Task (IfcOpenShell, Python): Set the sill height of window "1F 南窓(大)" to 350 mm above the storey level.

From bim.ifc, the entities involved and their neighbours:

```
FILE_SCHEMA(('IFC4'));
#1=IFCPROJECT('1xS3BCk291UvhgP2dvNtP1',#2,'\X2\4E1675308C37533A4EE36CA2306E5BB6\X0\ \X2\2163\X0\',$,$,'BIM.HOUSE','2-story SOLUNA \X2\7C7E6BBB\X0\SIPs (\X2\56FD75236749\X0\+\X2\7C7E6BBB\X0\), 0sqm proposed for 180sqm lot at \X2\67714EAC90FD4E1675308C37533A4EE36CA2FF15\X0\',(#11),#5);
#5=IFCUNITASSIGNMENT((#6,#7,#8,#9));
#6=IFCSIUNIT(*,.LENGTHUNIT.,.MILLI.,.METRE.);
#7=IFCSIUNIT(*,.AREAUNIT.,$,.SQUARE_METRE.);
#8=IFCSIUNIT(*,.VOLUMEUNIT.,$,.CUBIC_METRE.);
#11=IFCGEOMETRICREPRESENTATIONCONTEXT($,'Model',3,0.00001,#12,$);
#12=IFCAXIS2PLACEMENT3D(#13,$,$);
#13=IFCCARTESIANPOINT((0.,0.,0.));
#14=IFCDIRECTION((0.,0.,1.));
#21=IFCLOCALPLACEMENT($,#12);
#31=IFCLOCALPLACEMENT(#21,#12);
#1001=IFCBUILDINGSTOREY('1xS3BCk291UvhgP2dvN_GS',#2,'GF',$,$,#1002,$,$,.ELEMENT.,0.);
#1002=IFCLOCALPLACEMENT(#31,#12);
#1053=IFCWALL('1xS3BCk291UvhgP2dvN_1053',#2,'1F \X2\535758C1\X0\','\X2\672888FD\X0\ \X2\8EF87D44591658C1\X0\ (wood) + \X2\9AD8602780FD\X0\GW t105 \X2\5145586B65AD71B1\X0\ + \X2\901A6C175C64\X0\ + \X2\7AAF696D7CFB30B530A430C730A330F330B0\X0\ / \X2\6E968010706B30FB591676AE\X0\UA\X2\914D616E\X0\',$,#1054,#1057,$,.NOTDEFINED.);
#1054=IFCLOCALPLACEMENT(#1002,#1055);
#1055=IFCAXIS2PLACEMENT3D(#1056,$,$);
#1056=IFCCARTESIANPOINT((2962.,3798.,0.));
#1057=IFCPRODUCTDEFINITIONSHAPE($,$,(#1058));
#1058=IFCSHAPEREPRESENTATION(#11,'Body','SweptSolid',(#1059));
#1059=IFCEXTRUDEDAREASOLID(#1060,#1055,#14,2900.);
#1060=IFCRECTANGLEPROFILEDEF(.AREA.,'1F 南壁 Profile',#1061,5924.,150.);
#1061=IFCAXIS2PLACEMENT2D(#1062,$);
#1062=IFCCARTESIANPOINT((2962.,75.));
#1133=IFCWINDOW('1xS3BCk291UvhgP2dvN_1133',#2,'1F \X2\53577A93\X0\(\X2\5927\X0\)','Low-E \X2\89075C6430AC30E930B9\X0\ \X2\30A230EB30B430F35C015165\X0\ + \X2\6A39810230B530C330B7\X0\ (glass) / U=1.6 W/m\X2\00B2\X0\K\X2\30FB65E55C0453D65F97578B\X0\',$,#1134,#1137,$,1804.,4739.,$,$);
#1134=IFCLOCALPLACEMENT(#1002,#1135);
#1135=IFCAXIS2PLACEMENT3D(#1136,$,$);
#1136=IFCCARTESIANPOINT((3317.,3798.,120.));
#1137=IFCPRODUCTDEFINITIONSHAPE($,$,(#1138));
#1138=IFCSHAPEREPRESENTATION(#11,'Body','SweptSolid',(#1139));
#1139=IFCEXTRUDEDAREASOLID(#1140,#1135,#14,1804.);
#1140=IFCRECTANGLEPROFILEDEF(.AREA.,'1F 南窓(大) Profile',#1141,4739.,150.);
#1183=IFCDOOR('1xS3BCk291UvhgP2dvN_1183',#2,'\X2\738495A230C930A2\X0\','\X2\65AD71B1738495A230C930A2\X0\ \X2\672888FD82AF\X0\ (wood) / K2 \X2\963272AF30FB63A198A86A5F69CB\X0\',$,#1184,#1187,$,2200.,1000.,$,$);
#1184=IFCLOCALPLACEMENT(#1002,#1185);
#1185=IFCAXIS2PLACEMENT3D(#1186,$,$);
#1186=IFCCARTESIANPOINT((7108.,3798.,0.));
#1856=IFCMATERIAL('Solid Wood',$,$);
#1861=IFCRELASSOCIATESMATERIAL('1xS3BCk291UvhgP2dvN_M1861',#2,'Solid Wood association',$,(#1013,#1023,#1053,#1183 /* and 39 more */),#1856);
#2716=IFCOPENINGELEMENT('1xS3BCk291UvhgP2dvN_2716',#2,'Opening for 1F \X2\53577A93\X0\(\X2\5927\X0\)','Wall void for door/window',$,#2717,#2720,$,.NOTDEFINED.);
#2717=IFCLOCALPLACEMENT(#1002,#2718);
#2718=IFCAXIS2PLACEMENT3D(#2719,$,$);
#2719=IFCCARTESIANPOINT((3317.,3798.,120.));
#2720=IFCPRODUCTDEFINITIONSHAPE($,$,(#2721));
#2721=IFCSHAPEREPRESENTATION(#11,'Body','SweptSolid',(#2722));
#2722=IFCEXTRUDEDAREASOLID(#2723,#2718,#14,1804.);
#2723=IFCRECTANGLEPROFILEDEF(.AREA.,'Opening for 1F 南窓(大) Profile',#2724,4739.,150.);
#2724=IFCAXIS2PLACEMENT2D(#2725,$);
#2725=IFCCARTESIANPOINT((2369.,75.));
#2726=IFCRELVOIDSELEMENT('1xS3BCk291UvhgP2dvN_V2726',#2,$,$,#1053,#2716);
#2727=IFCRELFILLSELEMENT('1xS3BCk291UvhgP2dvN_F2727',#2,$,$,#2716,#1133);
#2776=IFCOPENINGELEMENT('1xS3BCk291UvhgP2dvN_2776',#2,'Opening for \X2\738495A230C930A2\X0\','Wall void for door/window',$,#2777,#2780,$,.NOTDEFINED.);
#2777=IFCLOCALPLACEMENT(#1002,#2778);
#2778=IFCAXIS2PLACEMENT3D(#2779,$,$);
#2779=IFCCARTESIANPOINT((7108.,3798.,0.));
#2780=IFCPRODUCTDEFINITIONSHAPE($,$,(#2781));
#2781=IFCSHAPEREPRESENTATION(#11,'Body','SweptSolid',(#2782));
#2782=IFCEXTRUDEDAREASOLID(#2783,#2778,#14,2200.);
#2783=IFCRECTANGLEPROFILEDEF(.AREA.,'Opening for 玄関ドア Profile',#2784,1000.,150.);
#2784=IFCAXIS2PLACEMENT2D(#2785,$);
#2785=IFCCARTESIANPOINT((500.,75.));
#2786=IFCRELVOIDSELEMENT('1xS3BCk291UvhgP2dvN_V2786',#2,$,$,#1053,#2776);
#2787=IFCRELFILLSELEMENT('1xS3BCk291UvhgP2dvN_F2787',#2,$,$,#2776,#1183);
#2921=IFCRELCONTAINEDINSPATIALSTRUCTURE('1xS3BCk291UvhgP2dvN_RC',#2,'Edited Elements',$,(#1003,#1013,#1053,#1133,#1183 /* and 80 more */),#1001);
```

```python
import numpy as np
import ifcopenshell
import ifcopenshell.api.geometry
import ifcopenshell.geom
import ifcopenshell.util.element
import ifcopenshell.util.placement
import ifcopenshell.util.shape
import ifcopenshell.util.unit

model = ifcopenshell.open("bim.ifc")
unit_scale = ifcopenshell.util.unit.calculate_unit_scale(model)

window = model.by_guid("1xS3BCk291UvhgP2dvN_1133")
opening = window.FillsVoids[0].RelatingOpeningElement
storey = ifcopenshell.util.element.get_container(window, ifc_class="IfcBuildingStorey")
level = ifcopenshell.util.placement.get_local_placement(storey.ObjectPlacement)[2, 3]

# The opening's origin need not be at the sill, so measure its lowest point.
shape = ifcopenshell.geom.create_shape(ifcopenshell.geom.settings(), opening)
bottom = ifcopenshell.util.shape.get_shape_bottom_elevation(shape, shape.geometry) / unit_scale
dz = level + 0.35 / unit_scale - bottom

shift = np.array([0.0, 0.0, dz])
# The window is not placed relative to its opening, so move both.
for product in (opening, window):
    matrix = ifcopenshell.util.placement.get_local_placement(product.ObjectPlacement)
    matrix[:3, 3] += shift
    ifcopenshell.api.geometry.edit_object_placement(model, product=product, matrix=matrix, is_si=False)

print(f"moved by {dz * unit_scale:+.3f} m")

model.write("bim_edited.ifc")
```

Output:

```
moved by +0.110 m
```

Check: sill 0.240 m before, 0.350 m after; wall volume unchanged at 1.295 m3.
